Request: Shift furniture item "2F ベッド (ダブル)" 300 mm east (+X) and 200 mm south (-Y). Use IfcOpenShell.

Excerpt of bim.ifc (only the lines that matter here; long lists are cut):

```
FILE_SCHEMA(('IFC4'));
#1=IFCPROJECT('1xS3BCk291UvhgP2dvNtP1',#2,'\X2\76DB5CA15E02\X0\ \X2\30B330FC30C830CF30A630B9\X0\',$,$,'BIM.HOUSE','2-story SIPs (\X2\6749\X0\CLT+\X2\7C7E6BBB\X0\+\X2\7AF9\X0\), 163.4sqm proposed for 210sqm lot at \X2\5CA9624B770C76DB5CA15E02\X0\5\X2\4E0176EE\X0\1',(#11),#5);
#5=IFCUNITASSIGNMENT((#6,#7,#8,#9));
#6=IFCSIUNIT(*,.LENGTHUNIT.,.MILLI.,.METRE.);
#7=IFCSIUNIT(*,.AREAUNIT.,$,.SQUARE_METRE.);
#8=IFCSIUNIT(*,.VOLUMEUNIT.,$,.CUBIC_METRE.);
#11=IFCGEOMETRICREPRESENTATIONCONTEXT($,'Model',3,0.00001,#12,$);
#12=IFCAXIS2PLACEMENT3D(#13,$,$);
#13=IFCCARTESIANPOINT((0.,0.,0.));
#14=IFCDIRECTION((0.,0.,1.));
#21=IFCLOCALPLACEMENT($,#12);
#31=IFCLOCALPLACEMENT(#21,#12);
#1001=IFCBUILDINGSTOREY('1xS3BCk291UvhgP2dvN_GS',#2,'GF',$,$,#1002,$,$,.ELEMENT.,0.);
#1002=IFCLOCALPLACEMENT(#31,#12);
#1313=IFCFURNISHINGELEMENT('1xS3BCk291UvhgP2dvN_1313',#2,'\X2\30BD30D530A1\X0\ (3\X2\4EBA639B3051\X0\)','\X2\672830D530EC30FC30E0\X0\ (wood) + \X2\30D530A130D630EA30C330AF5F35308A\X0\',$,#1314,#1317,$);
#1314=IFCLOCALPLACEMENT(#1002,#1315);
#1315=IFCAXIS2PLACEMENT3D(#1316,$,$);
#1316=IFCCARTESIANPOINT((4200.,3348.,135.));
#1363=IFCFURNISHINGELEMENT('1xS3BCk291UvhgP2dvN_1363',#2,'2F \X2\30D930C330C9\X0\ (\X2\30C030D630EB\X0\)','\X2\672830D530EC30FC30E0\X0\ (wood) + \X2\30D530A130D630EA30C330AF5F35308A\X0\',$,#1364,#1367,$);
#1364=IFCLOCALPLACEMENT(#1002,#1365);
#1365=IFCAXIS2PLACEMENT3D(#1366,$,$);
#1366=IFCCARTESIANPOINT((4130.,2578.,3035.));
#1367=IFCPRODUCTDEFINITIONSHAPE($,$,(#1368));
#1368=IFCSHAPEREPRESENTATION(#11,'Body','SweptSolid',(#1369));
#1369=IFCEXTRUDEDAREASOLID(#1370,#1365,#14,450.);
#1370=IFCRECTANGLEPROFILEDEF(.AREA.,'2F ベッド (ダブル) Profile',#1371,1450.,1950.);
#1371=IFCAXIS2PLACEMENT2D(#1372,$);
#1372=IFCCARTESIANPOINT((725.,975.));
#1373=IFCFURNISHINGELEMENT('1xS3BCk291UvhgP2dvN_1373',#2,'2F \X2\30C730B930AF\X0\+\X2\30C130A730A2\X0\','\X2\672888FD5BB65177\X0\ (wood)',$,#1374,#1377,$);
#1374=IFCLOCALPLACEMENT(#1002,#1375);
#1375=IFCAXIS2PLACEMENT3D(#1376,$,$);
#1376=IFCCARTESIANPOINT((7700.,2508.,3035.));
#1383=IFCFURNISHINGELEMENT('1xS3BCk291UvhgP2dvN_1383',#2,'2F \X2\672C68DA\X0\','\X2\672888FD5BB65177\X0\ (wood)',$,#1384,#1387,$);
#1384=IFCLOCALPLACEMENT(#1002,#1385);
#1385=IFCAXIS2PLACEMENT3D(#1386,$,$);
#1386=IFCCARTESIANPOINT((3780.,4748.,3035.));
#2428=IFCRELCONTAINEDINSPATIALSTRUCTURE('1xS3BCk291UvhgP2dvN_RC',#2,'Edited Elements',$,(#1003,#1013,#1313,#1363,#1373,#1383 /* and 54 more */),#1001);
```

```python
import ifcopenshell
import ifcopenshell.api.geometry
import ifcopenshell.util.placement

model = ifcopenshell.open("bim.ifc")

item = model.by_guid("1xS3BCk291UvhgP2dvN_1363")
matrix = ifcopenshell.util.placement.get_local_placement(item.ObjectPlacement)
matrix[0, 3] += 300.0
matrix[1, 3] -= 200.0
ifcopenshell.api.geometry.edit_object_placement(model, product=item, matrix=matrix, is_si=False)

print(ifcopenshell.util.placement.get_local_placement(item.ObjectPlacement).round(3) + 0.0)

model.write("bim-out.ifc")
```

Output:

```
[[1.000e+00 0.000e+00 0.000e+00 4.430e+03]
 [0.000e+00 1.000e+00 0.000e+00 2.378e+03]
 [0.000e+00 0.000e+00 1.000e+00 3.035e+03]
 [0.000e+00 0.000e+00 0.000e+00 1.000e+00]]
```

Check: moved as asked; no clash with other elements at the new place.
